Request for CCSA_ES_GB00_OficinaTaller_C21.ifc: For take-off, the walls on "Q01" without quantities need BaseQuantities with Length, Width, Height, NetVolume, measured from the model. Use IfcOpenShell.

First a look at what the model holds.

```python
import ifcopenshell
import ifcopenshell.util.element
import ifcopenshell.util.unit

model = ifcopenshell.open("CCSA_ES_GB00_OficinaTaller_C21.ifc")
print(model.schema)
for unit_type in ("LENGTHUNIT", "AREAUNIT", "VOLUMEUNIT"):
    print(unit_type, ifcopenshell.util.unit.calculate_unit_scale(model, unit_type))
storey = next(s for s in model.by_type("IfcBuildingStorey") if s.Name == "Q01")
walls = [e for e in ifcopenshell.util.element.get_decomposition(storey) if e.is_a("IfcWall")]
for e in sorted(walls, key=lambda e: e.id()):
    print(e.id(), e.is_a(), e.Name, list(ifcopenshell.util.element.get_psets(e, qtos_only=True)), sep=" | ")
```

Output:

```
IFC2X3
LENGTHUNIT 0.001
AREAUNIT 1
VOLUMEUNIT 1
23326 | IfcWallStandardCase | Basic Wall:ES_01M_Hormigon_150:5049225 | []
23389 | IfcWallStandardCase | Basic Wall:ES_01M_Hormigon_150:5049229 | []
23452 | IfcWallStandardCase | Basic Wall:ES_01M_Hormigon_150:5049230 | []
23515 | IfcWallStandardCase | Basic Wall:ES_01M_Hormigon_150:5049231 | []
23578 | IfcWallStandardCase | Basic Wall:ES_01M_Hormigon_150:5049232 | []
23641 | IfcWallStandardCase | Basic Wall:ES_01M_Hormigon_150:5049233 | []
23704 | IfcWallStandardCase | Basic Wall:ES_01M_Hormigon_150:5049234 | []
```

```python
import ifcopenshell
import ifcopenshell.api.pset
import ifcopenshell.geom
import ifcopenshell.util.element
import ifcopenshell.util.shape
import ifcopenshell.util.unit

model = ifcopenshell.open("CCSA_ES_GB00_OficinaTaller_C21.ifc")
unit_scale = ifcopenshell.util.unit.calculate_unit_scale(model)
volume_scale = ifcopenshell.util.unit.calculate_unit_scale(model, "VOLUMEUNIT")
settings = ifcopenshell.geom.settings()

storey = next(s for s in model.by_type("IfcBuildingStorey") if s.Name == "Q01")
walls = [e for e in ifcopenshell.util.element.get_decomposition(storey) if e.is_a("IfcWall")]

for e in sorted(walls, key=lambda e: e.id()):
    if ifcopenshell.util.element.get_psets(e, qtos_only=True, should_inherit=False):
        continue
    # Geometry comes back in metres, in the element's own axes.
    shape = ifcopenshell.geom.create_shape(settings, e)
    values = {
        "Length": ifcopenshell.util.shape.get_x(shape.geometry) / unit_scale,
        "Width": ifcopenshell.util.shape.get_y(shape.geometry) / unit_scale,
        "Height": ifcopenshell.util.shape.get_z(shape.geometry) / unit_scale,
        "NetVolume": ifcopenshell.util.shape.get_volume(shape.geometry) / volume_scale,
    }
    qto = ifcopenshell.api.pset.add_qto(model, product=e, name="BaseQuantities")
    ifcopenshell.api.pset.edit_qto(model, qto=qto, properties=values)
    print(e.id(), {k: round(v, 3) for k, v in values.items()})

model.write("CCSA_ES_GB00_OficinaTaller_C21_v2.ifc")
```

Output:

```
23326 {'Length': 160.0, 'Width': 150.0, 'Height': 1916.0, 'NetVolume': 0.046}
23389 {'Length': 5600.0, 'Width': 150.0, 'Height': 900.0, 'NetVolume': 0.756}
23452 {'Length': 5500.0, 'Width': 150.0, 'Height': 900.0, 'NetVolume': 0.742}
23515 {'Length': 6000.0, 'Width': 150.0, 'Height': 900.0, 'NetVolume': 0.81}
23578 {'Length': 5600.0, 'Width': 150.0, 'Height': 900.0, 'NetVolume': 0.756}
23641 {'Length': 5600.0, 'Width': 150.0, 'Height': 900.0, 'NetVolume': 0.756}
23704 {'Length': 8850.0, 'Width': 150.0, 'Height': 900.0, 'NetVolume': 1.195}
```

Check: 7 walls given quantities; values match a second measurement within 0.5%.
